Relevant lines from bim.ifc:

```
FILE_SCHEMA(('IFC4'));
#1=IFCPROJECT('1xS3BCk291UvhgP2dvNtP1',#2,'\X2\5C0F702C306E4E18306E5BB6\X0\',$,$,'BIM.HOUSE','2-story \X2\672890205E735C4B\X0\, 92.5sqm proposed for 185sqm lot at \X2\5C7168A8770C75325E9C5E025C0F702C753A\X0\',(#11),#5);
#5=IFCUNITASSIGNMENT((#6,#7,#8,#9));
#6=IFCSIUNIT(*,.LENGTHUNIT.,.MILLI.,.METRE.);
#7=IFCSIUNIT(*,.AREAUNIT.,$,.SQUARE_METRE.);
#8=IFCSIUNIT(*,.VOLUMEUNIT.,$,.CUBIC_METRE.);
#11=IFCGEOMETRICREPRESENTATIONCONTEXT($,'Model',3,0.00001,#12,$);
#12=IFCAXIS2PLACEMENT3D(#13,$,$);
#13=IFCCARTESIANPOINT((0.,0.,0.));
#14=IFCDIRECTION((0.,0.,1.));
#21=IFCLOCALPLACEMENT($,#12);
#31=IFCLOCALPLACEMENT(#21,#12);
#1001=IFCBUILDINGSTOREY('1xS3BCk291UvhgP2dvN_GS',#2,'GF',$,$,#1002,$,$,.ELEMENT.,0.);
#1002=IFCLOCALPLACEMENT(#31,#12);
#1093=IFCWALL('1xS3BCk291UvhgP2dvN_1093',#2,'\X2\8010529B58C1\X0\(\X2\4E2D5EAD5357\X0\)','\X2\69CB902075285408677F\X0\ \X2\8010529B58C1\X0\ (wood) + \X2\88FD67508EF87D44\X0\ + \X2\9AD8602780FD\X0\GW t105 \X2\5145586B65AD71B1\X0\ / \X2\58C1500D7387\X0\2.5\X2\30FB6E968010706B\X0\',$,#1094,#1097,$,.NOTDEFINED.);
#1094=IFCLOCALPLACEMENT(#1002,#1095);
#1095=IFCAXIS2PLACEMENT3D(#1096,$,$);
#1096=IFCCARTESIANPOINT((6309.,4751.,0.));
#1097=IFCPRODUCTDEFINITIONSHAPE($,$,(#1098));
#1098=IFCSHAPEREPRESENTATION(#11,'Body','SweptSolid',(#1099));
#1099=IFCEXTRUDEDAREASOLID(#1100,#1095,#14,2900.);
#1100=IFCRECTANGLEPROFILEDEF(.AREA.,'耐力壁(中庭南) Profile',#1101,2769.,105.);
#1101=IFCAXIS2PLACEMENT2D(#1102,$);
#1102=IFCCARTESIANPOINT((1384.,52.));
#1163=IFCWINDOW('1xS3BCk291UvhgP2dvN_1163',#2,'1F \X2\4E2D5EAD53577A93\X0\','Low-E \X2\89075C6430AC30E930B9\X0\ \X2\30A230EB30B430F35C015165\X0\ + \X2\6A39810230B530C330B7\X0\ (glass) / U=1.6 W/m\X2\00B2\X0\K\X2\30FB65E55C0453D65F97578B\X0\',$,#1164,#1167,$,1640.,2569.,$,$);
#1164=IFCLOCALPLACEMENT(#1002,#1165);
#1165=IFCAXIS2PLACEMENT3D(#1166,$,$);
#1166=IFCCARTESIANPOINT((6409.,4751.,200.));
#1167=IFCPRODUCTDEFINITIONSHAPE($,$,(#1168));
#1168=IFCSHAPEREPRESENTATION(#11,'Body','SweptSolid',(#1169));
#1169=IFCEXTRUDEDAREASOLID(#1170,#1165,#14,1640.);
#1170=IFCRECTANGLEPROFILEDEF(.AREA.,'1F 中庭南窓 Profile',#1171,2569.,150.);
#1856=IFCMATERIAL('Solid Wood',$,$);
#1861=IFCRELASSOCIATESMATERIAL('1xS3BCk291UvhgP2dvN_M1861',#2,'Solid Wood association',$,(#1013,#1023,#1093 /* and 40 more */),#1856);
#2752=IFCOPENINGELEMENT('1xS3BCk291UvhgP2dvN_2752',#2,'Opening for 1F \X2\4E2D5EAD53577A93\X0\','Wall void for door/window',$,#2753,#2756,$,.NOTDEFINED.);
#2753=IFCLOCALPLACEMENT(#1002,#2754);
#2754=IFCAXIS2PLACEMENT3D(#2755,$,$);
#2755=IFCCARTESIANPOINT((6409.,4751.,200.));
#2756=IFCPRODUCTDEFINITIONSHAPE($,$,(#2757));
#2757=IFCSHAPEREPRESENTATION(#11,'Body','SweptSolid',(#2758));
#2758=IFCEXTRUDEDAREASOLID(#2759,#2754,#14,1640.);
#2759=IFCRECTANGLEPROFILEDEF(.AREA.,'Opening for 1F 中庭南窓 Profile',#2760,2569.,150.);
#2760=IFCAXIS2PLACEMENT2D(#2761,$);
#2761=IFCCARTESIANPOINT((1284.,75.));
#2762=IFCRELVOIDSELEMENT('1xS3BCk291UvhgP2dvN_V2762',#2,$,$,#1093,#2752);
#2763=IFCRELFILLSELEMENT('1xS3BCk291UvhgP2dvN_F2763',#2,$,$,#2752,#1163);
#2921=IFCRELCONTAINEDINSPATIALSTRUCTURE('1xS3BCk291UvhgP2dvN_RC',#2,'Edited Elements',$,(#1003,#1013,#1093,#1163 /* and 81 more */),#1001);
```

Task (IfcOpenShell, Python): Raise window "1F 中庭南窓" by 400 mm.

```python
import numpy as np
import ifcopenshell
import ifcopenshell.api.geometry
import ifcopenshell.util.placement
import ifcopenshell.util.unit

model = ifcopenshell.open("bim.ifc")
unit_scale = ifcopenshell.util.unit.calculate_unit_scale(model)

window = model.by_guid("1xS3BCk291UvhgP2dvN_1163")
opening = window.FillsVoids[0].RelatingOpeningElement
dz = 400.0

shift = np.array([0.0, 0.0, dz])
# The window is not placed relative to its opening, so move both.
for product in (opening, window):
    matrix = ifcopenshell.util.placement.get_local_placement(product.ObjectPlacement)
    matrix[:3, 3] += shift
    ifcopenshell.api.geometry.edit_object_placement(model, product=product, matrix=matrix, is_si=False)

print(f"moved by {dz * unit_scale:+.3f} m")

model.write("bim_rev.ifc")
```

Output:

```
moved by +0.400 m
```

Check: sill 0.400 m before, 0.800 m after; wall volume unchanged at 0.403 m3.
